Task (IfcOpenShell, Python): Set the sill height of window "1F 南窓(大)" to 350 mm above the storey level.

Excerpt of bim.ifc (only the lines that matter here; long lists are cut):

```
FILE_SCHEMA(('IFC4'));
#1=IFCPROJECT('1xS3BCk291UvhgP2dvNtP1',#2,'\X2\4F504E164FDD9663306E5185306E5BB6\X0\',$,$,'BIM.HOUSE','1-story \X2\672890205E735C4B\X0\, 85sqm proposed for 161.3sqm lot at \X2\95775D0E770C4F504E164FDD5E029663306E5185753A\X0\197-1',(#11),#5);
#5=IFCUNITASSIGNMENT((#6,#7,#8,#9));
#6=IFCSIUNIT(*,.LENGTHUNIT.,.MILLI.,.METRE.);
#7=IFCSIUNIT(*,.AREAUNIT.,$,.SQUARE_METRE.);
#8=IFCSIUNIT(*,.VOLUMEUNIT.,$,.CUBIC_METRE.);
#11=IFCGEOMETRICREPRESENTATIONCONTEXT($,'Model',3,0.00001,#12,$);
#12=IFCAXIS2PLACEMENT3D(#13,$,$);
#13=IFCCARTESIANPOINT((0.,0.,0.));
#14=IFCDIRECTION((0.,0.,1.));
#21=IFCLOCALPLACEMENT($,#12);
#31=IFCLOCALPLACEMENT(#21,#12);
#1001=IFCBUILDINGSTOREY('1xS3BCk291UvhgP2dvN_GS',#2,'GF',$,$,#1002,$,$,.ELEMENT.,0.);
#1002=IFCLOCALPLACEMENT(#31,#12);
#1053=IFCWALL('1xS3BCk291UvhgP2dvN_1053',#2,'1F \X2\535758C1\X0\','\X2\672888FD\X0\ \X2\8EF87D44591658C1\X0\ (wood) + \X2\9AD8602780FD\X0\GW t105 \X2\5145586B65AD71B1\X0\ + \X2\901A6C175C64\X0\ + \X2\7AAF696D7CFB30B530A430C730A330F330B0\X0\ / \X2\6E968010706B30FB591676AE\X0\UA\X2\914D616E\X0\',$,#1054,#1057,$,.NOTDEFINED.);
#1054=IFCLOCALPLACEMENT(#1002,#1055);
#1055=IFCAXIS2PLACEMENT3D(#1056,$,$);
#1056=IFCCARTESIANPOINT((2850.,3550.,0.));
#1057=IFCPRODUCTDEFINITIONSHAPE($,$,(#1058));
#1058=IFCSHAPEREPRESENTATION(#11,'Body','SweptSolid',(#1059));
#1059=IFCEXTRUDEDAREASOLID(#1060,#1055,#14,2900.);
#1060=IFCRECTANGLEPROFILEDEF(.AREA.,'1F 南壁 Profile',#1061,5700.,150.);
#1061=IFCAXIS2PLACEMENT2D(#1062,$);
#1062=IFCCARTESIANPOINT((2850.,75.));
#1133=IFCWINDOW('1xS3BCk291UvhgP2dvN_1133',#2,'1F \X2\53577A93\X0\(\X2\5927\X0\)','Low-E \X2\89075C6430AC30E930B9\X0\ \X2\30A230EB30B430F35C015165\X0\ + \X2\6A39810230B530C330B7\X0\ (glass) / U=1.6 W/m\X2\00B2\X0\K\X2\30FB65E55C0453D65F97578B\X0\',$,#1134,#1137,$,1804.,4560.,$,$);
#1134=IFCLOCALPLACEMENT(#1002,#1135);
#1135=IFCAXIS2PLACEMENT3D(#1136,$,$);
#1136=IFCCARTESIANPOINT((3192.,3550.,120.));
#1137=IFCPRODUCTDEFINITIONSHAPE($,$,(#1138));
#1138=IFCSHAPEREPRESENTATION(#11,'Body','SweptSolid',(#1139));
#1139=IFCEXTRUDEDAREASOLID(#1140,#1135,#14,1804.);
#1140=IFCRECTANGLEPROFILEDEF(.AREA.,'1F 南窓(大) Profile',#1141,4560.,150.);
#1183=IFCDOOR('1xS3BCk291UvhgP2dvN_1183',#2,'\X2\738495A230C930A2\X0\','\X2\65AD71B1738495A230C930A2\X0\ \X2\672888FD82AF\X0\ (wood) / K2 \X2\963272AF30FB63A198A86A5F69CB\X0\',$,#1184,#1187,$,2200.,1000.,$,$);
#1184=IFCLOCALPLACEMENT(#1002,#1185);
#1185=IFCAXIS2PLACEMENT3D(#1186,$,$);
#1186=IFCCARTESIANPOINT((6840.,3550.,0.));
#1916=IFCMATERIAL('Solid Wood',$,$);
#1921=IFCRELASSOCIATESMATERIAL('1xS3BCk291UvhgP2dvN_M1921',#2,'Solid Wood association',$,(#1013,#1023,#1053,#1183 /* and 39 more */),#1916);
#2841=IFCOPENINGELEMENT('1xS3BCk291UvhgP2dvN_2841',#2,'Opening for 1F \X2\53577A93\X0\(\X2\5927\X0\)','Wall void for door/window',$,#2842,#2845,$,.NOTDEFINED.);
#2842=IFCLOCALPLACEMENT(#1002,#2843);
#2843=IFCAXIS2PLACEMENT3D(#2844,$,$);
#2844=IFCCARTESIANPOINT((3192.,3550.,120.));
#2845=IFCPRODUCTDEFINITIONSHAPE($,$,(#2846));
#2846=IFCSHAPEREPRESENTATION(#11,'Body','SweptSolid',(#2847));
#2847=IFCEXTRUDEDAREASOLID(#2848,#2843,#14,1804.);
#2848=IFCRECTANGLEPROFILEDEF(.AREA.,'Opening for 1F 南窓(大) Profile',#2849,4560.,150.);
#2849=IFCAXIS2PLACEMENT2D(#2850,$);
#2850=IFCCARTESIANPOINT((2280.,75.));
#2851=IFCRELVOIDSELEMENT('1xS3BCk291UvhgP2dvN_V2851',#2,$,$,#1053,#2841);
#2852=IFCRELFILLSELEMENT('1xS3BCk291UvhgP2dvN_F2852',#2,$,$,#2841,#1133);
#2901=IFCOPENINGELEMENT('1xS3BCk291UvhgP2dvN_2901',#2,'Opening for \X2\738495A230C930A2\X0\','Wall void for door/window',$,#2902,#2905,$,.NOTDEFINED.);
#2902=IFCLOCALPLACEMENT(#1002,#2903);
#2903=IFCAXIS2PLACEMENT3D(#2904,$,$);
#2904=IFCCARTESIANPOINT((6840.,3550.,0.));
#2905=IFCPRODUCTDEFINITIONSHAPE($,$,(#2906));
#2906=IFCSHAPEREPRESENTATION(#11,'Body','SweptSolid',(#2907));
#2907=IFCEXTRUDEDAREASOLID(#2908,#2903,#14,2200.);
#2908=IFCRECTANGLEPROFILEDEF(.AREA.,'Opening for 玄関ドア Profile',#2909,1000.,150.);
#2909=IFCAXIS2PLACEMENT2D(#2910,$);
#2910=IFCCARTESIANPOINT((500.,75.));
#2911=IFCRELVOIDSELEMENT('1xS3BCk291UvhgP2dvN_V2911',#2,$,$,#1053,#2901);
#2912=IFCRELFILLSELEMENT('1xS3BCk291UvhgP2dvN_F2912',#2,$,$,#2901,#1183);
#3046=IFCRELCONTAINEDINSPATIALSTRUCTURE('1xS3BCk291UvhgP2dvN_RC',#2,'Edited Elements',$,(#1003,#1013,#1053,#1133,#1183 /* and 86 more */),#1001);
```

```python
import numpy as np
import ifcopenshell
import ifcopenshell.api.geometry
import ifcopenshell.geom
import ifcopenshell.util.element
import ifcopenshell.util.placement
import ifcopenshell.util.shape
import ifcopenshell.util.unit

model = ifcopenshell.open("bim.ifc")
unit_scale = ifcopenshell.util.unit.calculate_unit_scale(model)

window = model.by_guid("1xS3BCk291UvhgP2dvN_1133")
opening = window.FillsVoids[0].RelatingOpeningElement
storey = ifcopenshell.util.element.get_container(window, ifc_class="IfcBuildingStorey")
level = ifcopenshell.util.placement.get_local_placement(storey.ObjectPlacement)[2, 3]

# The opening's origin need not be at the sill, so measure its lowest point.
shape = ifcopenshell.geom.create_shape(ifcopenshell.geom.settings(), opening)
bottom = ifcopenshell.util.shape.get_shape_bottom_elevation(shape, shape.geometry) / unit_scale
dz = level + 0.35 / unit_scale - bottom

shift = np.array([0.0, 0.0, dz])
# The window is not placed relative to its opening, so move both.
for product in (opening, window):
    matrix = ifcopenshell.util.placement.get_local_placement(product.ObjectPlacement)
    matrix[:3, 3] += shift
    ifcopenshell.api.geometry.edit_object_placement(model, product=product, matrix=matrix, is_si=False)

print(f"moved by {dz * unit_scale:+.3f} m")

model.write("bim_updated.ifc")
```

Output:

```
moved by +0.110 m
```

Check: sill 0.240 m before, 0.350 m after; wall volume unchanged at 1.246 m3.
